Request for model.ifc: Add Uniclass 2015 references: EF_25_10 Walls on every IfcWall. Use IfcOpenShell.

First a look at what the model holds.

```python
import ifcopenshell

model = ifcopenshell.open("model.ifc")
print(model.schema)
print("classifications:", [c.Name for c in model.by_type("IfcClassification")])
for ifc_class in ("IfcDoor", "IfcRoof", "IfcStair", "IfcWall", "IfcWindow"):
    print(ifc_class, len(model.by_type(ifc_class)))
```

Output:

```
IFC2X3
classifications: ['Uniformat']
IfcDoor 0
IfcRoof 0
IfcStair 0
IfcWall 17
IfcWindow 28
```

```python
import ifcopenshell
import ifcopenshell.api.classification

model = ifcopenshell.open("model.ifc")

# IFC2X3 requires Source and Edition and has no link from the project to the system.
system = model.create_entity("IfcClassification", Source="NBS", Edition="2015", Name="Uniclass 2015")

codes = {
    "IfcWall": ("EF_25_10", "Walls"),
}
for ifc_class, (code, name) in codes.items():
    products = model.by_type(ifc_class)
    ifcopenshell.api.classification.add_reference(
        model, products=products, classification=system, identification=code, name=name
    )
    print(code, len(products))

model.write("model-out.ifc")
```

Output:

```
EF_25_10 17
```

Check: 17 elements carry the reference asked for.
